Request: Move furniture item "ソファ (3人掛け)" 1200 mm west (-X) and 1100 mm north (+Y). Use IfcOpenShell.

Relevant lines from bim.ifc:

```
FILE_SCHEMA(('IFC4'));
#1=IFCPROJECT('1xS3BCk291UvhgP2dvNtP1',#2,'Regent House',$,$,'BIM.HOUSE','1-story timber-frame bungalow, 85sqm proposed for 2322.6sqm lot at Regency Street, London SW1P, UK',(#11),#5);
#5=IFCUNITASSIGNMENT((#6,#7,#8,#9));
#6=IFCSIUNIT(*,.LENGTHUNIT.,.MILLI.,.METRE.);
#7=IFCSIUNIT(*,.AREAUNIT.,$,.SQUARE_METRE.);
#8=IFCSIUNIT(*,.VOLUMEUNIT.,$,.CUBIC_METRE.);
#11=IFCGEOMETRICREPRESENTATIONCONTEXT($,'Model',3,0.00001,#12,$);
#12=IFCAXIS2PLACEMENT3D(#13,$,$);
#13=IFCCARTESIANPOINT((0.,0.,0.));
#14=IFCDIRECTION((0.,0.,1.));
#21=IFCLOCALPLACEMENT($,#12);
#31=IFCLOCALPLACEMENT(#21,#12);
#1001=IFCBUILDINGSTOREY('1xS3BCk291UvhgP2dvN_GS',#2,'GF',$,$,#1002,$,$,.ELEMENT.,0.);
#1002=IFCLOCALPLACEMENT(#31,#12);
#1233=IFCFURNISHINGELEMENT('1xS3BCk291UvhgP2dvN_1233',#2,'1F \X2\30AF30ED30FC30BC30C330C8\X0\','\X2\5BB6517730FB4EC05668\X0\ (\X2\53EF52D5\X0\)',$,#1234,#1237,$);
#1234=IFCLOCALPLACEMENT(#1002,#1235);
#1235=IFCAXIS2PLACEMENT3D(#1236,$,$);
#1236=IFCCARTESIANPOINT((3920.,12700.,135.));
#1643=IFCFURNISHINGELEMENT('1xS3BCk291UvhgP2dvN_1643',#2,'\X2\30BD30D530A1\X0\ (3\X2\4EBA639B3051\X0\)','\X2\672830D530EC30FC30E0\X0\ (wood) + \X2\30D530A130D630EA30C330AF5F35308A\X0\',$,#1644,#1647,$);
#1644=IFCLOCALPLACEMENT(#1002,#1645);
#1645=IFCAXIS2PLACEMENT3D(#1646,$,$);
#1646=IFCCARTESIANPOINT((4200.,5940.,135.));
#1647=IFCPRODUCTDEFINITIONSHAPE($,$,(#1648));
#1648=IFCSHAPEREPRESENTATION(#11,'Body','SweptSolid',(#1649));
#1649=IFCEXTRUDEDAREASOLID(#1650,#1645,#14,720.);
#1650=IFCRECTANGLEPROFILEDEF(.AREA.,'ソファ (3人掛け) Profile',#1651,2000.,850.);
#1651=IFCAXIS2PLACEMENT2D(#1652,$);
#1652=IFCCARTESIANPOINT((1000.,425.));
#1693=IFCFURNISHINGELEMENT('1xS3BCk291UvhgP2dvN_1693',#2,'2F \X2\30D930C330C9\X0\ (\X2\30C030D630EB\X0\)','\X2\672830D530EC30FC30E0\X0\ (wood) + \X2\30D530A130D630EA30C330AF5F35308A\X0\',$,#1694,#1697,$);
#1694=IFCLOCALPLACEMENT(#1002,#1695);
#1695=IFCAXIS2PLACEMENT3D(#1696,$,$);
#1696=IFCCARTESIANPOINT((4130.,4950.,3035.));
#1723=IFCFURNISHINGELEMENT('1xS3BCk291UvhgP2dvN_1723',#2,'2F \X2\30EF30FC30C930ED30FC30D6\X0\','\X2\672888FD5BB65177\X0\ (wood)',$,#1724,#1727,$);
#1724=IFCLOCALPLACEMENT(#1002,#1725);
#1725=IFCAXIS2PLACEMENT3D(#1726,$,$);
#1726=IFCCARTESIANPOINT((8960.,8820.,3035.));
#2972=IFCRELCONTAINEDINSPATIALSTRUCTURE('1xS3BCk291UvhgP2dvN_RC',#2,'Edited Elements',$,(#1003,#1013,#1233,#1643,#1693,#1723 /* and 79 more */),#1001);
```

```python
import ifcopenshell
import ifcopenshell.api.geometry
import ifcopenshell.util.placement
import ifcopenshell.util.unit

model = ifcopenshell.open("bim.ifc")
unit_scale = ifcopenshell.util.unit.calculate_unit_scale(model)

item = model.by_id(1643)
matrix = ifcopenshell.util.placement.get_local_placement(item.ObjectPlacement)
matrix[0, 3] -= 1.2 / unit_scale
matrix[1, 3] += 1.1 / unit_scale
ifcopenshell.api.geometry.edit_object_placement(model, product=item, matrix=matrix, is_si=False)

print(ifcopenshell.util.placement.get_local_placement(item.ObjectPlacement).round(3) + 0.0)

model.write("bim_updated.ifc")
```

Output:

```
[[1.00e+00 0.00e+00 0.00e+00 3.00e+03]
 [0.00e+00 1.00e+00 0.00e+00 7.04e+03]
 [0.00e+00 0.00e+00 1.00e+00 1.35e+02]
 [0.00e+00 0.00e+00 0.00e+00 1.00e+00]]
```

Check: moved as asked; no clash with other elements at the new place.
